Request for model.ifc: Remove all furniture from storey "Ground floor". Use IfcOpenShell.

First a look at what the model holds.

```python
import ifcopenshell
import ifcopenshell.util.element

model = ifcopenshell.open("model.ifc")
print(model.schema)
storey = next(s for s in model.by_type("IfcBuildingStorey") if s.Name == "Ground floor")
furniture = [e for e in ifcopenshell.util.element.get_decomposition(storey) if e.is_a("IfcFurnishingElement")]
seen = {}
for e in furniture:
    element_type = ifcopenshell.util.element.get_type(e)
    name = element_type.Name if element_type not in (None, e) else None
    seen[name] = seen.get(name, 0) + 1
for name, count in sorted(seen.items(), key=str):
    print(count, "x", name)
```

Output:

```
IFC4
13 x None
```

```python
import ifcopenshell
import ifcopenshell.api.root
import ifcopenshell.util.element

model = ifcopenshell.open("model.ifc")

storey = next(s for s in model.by_type("IfcBuildingStorey") if s.Name == "Ground floor")
furniture = [e for e in ifcopenshell.util.element.get_decomposition(storey) if e.is_a("IfcFurnishingElement")]

for e in furniture:
    ifcopenshell.api.root.remove_product(model, product=e)
print(len(furniture), "removed")

model.write("model_rev.ifc")
```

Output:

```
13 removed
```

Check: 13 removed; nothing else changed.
